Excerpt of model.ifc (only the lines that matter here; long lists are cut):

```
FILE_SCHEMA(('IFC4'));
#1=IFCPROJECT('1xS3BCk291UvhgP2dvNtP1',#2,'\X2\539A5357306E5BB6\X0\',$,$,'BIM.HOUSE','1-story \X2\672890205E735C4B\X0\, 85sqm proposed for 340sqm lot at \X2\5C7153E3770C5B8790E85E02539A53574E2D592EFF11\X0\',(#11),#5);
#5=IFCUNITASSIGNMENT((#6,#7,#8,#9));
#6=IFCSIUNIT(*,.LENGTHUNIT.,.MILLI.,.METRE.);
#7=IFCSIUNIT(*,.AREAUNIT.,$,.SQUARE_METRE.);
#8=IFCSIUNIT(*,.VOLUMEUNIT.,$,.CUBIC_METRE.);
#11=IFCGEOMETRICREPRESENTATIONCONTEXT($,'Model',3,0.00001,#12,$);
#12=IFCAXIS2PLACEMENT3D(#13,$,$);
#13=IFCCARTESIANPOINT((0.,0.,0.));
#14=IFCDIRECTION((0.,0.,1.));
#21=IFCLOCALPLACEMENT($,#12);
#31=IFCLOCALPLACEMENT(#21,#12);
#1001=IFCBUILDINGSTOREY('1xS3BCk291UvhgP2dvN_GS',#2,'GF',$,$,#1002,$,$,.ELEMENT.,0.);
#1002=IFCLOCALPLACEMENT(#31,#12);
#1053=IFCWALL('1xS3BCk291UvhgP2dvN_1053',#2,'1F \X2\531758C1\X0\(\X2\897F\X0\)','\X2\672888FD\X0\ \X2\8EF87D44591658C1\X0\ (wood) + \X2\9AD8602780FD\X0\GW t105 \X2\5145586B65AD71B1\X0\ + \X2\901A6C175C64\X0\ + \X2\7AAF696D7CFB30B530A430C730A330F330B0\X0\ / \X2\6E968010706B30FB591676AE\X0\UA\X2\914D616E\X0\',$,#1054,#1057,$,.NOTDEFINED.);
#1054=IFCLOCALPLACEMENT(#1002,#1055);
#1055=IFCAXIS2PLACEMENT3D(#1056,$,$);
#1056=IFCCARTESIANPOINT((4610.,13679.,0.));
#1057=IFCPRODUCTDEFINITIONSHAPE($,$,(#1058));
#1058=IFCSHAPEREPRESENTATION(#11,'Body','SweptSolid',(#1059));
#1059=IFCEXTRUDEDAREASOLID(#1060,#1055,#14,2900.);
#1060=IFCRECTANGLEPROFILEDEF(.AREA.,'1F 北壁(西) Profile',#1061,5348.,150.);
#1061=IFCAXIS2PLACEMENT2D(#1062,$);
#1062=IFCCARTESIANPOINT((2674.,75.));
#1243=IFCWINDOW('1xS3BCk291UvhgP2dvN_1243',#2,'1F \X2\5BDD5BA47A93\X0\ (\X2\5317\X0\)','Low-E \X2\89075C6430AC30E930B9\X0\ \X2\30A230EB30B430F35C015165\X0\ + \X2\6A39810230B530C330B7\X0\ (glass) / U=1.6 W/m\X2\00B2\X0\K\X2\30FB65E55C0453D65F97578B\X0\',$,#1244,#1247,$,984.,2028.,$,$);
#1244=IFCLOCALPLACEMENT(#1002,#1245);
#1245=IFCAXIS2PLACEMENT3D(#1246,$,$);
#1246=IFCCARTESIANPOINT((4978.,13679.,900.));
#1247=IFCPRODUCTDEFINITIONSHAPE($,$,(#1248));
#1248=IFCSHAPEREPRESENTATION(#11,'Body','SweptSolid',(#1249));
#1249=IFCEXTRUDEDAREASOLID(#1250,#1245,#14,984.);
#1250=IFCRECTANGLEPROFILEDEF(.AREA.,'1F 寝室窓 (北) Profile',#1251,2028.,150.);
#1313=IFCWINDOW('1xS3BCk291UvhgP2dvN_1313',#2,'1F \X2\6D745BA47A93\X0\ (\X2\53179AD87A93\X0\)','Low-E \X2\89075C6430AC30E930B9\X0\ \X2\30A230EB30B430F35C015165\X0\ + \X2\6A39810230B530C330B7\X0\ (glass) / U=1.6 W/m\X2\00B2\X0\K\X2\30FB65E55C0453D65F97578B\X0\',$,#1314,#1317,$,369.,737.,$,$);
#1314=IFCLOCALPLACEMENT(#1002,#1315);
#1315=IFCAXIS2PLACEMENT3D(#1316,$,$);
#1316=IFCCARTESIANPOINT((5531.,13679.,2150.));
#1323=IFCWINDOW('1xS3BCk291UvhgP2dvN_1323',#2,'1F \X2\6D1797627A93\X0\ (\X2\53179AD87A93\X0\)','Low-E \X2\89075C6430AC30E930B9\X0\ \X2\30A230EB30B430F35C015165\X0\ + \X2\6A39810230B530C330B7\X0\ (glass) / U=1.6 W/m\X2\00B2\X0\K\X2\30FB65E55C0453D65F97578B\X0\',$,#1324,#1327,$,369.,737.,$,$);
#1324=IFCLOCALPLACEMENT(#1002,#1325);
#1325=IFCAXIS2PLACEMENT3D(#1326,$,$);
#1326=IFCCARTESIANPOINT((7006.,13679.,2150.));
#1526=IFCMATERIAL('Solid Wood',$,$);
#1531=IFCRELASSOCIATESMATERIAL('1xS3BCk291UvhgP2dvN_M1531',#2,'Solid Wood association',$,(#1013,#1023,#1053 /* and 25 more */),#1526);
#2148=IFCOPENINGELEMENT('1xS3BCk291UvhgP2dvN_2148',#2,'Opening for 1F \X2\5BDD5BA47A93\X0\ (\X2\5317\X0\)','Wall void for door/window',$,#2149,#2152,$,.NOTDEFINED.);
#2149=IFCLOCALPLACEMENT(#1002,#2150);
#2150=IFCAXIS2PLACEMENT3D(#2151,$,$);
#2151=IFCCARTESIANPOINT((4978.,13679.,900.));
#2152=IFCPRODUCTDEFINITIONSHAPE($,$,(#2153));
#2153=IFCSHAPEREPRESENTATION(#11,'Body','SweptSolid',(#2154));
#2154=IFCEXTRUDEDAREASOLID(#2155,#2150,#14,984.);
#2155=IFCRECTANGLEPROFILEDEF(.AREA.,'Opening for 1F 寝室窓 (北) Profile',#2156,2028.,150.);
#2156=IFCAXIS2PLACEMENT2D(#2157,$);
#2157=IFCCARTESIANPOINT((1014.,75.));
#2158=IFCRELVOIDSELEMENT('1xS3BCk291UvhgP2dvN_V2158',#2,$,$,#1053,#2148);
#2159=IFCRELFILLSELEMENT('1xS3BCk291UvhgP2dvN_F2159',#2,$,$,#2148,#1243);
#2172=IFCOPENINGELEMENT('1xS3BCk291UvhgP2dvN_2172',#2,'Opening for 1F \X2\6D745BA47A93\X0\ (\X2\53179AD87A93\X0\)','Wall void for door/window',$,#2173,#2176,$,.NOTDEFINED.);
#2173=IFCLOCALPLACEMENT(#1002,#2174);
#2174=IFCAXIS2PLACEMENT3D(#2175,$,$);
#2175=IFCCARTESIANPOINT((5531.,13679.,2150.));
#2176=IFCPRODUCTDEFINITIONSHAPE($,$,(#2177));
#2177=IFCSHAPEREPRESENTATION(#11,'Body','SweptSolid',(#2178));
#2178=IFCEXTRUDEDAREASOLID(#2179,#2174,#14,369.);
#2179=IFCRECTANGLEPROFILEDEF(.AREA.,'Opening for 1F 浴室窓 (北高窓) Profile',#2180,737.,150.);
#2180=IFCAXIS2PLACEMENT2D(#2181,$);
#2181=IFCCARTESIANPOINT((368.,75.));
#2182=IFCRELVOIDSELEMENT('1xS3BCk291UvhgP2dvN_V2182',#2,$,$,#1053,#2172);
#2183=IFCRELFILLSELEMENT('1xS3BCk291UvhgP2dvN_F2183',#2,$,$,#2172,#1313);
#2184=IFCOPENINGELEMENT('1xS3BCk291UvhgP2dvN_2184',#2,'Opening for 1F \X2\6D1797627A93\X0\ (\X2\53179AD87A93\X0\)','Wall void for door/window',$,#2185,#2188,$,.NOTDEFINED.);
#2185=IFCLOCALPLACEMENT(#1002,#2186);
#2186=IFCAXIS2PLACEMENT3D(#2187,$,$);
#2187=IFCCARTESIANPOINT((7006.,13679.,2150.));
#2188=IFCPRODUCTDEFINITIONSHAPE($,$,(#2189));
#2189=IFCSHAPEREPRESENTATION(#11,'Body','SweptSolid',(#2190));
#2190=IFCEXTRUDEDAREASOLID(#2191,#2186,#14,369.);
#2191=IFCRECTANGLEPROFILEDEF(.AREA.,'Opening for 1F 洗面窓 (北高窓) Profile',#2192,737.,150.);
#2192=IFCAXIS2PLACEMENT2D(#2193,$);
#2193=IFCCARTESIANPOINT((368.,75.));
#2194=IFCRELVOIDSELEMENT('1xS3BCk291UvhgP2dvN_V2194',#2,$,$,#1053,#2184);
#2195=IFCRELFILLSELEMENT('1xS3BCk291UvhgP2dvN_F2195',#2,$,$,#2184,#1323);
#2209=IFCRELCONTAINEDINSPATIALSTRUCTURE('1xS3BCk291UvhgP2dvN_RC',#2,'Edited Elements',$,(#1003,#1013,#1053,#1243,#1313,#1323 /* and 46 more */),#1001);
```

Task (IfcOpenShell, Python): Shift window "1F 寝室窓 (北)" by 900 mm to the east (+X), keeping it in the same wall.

```python
import ifcopenshell
import ifcopenshell.api.geometry
import ifcopenshell.util.placement

model = ifcopenshell.open("model.ifc")

window = model.by_id(1243)
opening = window.FillsVoids[0].RelatingOpeningElement
wall = opening.VoidsElements[0].RelatingBuildingElement

wall_matrix = ifcopenshell.util.placement.get_local_placement(wall.ObjectPlacement)
shift = wall_matrix[:3, 0] * 900.0
before = ifcopenshell.util.placement.get_local_placement(window.ObjectPlacement)[:3, 3].copy()

# The window is not placed relative to its opening, so move both.
for product in (opening, window):
    matrix = ifcopenshell.util.placement.get_local_placement(product.ObjectPlacement)
    matrix[:3, 3] += shift
    ifcopenshell.api.geometry.edit_object_placement(model, product=product, matrix=matrix, is_si=False)

after = ifcopenshell.util.placement.get_local_placement(window.ObjectPlacement)[:3, 3]
print("window moved by", (after - before).round(3) + 0.0)

model.write("model_updated.ifc")
```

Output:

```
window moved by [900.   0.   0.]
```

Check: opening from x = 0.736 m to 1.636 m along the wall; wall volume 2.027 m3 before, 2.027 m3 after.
